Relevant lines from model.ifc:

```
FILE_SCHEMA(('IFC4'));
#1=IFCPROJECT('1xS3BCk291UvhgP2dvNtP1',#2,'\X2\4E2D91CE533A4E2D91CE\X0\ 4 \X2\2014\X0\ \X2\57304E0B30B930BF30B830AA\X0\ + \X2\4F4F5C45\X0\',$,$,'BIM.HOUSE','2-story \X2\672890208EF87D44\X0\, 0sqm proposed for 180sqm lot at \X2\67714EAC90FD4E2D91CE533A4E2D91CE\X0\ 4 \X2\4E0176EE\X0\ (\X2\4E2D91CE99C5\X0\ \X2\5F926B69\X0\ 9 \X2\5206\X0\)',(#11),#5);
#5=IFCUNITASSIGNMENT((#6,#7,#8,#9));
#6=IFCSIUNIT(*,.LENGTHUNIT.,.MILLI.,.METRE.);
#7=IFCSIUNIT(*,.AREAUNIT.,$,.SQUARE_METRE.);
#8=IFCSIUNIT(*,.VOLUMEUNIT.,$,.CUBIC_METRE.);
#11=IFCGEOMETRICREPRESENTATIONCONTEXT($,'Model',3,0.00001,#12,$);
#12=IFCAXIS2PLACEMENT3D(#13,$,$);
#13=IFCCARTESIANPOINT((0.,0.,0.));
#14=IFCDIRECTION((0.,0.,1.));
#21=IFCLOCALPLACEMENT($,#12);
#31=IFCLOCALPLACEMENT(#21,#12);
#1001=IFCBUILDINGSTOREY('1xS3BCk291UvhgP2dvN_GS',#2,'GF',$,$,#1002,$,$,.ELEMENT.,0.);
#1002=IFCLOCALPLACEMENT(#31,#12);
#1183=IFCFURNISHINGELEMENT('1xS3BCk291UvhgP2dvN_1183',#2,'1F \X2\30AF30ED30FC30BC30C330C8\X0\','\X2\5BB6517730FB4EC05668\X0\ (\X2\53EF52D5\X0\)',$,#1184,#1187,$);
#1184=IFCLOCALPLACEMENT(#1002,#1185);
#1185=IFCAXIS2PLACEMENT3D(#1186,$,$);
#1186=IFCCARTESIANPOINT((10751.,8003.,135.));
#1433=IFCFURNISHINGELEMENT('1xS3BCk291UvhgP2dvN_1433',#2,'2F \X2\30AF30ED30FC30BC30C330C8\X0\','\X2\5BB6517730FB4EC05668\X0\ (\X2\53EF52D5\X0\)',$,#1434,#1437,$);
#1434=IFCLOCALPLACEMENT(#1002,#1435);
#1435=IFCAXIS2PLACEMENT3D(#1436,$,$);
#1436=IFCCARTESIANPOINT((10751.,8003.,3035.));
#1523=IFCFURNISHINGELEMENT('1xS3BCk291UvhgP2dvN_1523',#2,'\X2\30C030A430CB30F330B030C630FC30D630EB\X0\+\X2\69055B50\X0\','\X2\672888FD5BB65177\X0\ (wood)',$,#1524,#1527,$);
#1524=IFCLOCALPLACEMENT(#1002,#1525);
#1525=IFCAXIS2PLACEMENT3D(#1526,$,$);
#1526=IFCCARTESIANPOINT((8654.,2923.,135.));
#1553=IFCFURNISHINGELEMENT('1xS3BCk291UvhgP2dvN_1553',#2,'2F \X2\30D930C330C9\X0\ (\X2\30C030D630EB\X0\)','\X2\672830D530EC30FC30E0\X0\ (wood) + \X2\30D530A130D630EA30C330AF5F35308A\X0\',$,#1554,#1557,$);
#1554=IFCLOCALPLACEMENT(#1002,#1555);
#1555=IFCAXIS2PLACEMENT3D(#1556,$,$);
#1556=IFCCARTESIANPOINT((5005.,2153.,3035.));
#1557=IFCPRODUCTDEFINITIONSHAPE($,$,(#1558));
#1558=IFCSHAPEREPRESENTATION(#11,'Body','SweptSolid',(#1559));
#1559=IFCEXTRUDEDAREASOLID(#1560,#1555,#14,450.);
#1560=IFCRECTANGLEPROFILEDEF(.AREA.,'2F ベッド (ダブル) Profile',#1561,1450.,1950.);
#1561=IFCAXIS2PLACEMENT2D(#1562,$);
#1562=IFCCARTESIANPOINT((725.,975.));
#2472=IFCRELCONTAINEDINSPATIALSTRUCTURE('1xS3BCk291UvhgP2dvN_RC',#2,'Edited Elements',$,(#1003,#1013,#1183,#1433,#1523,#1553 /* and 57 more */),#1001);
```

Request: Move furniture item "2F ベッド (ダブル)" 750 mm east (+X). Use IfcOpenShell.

```python
import ifcopenshell
import ifcopenshell.api.geometry
import ifcopenshell.util.placement
import ifcopenshell.util.unit

model = ifcopenshell.open("model.ifc")
unit_scale = ifcopenshell.util.unit.calculate_unit_scale(model)

item = model.by_guid("1xS3BCk291UvhgP2dvN_1553")
matrix = ifcopenshell.util.placement.get_local_placement(item.ObjectPlacement)
matrix[0, 3] += 0.75 / unit_scale
ifcopenshell.api.geometry.edit_object_placement(model, product=item, matrix=matrix, is_si=False)

print(ifcopenshell.util.placement.get_local_placement(item.ObjectPlacement).round(3) + 0.0)

model.write("model_v2.ifc")
```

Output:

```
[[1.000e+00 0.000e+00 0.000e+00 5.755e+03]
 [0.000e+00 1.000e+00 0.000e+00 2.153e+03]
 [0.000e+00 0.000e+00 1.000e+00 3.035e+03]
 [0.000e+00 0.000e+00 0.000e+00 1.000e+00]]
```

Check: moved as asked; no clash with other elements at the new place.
